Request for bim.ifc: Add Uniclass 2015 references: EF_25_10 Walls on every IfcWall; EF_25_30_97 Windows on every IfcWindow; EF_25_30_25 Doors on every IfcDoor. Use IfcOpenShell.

First a look at what the model holds.

```python
import ifcopenshell

model = ifcopenshell.open("bim.ifc")
print(model.schema)
print("classifications:", [c.Name for c in model.by_type("IfcClassification")])
for ifc_class in ("IfcDoor", "IfcRoof", "IfcStair", "IfcWall", "IfcWindow"):
    print(ifc_class, len(model.by_type(ifc_class)))
```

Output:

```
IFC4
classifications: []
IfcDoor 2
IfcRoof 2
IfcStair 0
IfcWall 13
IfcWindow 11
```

```python
import ifcopenshell
import ifcopenshell.api.classification

model = ifcopenshell.open("bim.ifc")

system = ifcopenshell.api.classification.add_classification(model, classification="Uniclass 2015")

codes = {
    "IfcWall": ("EF_25_10", "Walls"),
    "IfcWindow": ("EF_25_30_97", "Windows"),
    "IfcDoor": ("EF_25_30_25", "Doors"),
}
for ifc_class, (code, name) in codes.items():
    products = model.by_type(ifc_class)
    ifcopenshell.api.classification.add_reference(
        model, products=products, classification=system, identification=code, name=name
    )
    print(code, len(products))

model.write("bim_v2.ifc")
```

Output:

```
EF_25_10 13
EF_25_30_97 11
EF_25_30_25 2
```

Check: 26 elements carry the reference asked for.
